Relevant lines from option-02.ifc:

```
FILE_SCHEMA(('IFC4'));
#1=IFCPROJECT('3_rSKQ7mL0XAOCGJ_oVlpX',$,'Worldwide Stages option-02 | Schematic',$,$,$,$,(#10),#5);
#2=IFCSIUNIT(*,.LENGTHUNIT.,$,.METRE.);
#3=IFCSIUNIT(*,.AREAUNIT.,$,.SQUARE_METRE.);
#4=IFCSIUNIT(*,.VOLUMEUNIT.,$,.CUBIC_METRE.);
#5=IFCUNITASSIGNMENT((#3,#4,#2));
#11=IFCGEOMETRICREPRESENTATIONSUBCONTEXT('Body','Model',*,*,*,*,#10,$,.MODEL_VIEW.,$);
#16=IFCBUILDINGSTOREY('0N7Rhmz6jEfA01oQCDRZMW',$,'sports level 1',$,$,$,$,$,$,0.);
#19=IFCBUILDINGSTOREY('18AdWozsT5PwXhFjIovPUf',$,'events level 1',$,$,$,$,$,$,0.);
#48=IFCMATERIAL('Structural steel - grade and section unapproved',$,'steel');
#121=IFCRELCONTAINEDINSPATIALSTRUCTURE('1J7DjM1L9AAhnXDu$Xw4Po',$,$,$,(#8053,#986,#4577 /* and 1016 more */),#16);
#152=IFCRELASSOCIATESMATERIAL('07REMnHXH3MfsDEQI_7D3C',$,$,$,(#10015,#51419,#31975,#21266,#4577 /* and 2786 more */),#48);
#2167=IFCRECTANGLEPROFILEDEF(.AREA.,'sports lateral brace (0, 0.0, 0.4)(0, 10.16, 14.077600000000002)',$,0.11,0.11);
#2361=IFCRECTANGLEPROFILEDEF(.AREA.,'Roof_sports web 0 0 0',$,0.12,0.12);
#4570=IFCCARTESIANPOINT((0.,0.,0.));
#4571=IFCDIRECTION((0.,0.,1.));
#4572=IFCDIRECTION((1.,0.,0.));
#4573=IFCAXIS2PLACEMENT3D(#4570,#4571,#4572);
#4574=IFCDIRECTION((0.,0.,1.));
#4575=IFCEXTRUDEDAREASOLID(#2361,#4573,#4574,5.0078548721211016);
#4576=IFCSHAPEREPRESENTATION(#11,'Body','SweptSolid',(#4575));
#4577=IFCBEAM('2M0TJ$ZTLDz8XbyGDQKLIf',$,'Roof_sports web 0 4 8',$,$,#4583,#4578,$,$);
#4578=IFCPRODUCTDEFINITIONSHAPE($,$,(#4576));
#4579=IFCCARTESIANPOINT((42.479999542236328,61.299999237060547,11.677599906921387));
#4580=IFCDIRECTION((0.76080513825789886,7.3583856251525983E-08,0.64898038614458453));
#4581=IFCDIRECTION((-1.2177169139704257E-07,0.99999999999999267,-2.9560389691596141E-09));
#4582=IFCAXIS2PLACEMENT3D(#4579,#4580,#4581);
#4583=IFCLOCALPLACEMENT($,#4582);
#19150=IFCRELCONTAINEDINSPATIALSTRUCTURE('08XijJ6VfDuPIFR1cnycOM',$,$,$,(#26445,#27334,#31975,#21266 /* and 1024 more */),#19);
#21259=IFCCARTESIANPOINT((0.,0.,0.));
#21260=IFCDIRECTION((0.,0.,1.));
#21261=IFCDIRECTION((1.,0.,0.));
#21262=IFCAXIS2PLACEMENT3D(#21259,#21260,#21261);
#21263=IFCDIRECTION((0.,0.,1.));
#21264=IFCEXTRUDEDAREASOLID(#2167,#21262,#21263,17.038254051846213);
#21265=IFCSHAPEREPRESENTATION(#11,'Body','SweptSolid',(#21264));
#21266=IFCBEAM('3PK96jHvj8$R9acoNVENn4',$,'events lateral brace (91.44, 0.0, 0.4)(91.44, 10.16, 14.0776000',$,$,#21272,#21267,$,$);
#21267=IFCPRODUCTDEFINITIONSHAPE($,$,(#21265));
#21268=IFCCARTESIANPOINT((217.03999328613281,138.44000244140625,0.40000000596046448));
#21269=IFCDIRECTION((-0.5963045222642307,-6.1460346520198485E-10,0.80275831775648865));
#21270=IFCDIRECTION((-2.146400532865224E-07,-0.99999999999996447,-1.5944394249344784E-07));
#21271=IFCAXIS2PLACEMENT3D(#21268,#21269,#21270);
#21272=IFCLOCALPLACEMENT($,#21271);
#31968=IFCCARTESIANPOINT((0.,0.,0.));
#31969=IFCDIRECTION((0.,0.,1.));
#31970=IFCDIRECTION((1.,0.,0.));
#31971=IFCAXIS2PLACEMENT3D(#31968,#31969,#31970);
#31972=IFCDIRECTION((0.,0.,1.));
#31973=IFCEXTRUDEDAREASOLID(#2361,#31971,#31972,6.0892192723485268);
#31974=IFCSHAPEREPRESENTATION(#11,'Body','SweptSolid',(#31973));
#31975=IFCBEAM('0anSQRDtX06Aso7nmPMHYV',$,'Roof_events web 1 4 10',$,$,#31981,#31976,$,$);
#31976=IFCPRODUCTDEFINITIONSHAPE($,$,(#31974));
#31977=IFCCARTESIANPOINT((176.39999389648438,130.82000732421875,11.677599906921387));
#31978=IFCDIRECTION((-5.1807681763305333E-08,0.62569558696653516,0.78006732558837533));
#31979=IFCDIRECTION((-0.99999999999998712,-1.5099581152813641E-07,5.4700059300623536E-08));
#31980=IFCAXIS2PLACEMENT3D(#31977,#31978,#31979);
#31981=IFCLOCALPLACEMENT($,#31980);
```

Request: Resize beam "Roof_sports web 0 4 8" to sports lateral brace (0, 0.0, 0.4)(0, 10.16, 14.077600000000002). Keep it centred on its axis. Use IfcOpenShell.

```python
import ifcopenshell
import ifcopenshell.util.element
import ifcopenshell.util.representation

model = ifcopenshell.open("option-02.ifc")

member = model.by_guid("2M0TJ$ZTLDz8XbyGDQKLIf")
source = next(p for p in model.by_type("IfcRectangleProfileDef") if p.ProfileName == "sports lateral brace (0, 0.0, 0.4)(0, 10.16, 14.077600000000002)")

body = ifcopenshell.util.representation.get_representation(member, "Model", "Body")
solid = body.Items[0]
old_profile = solid.SweptArea

# Copy the section's sizes but keep this member's own profile position.
profile = ifcopenshell.util.element.copy(model, source)
profile.Position = old_profile.Position
solid.SweptArea = profile
if not model.get_total_inverses(old_profile):
    ifcopenshell.util.element.remove_deep2(model, old_profile)

print(solid.SweptArea)

model.write("option-02_v2.ifc")
```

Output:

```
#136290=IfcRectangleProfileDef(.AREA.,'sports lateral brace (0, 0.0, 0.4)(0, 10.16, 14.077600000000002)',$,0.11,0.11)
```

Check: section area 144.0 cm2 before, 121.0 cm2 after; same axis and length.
